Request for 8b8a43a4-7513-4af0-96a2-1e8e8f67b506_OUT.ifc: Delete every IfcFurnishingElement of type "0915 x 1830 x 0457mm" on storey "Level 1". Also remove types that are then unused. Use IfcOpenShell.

First a look at what the model holds.

```python
import ifcopenshell
import ifcopenshell.util.element

model = ifcopenshell.open("8b8a43a4-7513-4af0-96a2-1e8e8f67b506_OUT.ifc")
print(model.schema)
storey = next(s for s in model.by_type("IfcBuildingStorey") if s.Name == "Level 1")
furniture = [e for e in ifcopenshell.util.element.get_decomposition(storey) if e.is_a("IfcFurnishingElement")]
seen = {}
for e in furniture:
    element_type = ifcopenshell.util.element.get_type(e)
    name = element_type.Name if element_type not in (None, e) else None
    seen[name] = seen.get(name, 0) + 1
for name, count in sorted(seen.items(), key=str):
    print(count, "x", name)
```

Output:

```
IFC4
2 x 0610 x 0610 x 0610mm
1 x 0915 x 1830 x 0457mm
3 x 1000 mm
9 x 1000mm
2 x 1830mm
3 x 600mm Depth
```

```python
import ifcopenshell
import ifcopenshell.api.root
import ifcopenshell.util.element

model = ifcopenshell.open("8b8a43a4-7513-4af0-96a2-1e8e8f67b506_OUT.ifc")

storey = next(s for s in model.by_type("IfcBuildingStorey") if s.Name == "Level 1")
furniture = [e for e in ifcopenshell.util.element.get_decomposition(storey) if e.is_a("IfcFurnishingElement")]
targets = [e for e in furniture if (t := ifcopenshell.util.element.get_type(e)) not in (None, e) and t.Name == "0915 x 1830 x 0457mm"]
types = {ifcopenshell.util.element.get_type(e) for e in targets} - {None, *targets}

for e in targets:
    ifcopenshell.api.root.remove_product(model, product=e)
print(len(targets), "removed")

unused = [t for t in types if not ifcopenshell.util.element.get_types(t)]
for t in unused:
    ifcopenshell.api.root.remove_product(model, product=t)
print(len(unused), "unused types removed")

model.write("8b8a43a4-7513-4af0-96a2-1e8e8f67b506_OUT_edited.ifc")
```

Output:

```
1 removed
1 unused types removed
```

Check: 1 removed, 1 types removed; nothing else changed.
